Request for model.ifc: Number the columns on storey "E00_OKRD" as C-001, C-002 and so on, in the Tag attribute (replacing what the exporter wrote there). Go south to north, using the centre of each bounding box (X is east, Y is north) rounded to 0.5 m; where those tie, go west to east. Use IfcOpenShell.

First a look at what the model holds.

```python
import ifcopenshell
import ifcopenshell.util.element
import ifcopenshell.util.placement

model = ifcopenshell.open("model.ifc")
print(model.schema)
storey = next(s for s in model.by_type("IfcBuildingStorey") if s.Name == "E00_OKRD")
columns = [e for e in ifcopenshell.util.element.get_decomposition(storey) if e.is_a("IfcColumn")]
for e in sorted(columns, key=lambda e: e.id()):
    origin = ifcopenshell.util.placement.get_local_placement(e.ObjectPlacement)[:3, 3]
    print(e.id(), e.Tag, e.Name, origin.round(2) + 0.0, sep=" | ")
```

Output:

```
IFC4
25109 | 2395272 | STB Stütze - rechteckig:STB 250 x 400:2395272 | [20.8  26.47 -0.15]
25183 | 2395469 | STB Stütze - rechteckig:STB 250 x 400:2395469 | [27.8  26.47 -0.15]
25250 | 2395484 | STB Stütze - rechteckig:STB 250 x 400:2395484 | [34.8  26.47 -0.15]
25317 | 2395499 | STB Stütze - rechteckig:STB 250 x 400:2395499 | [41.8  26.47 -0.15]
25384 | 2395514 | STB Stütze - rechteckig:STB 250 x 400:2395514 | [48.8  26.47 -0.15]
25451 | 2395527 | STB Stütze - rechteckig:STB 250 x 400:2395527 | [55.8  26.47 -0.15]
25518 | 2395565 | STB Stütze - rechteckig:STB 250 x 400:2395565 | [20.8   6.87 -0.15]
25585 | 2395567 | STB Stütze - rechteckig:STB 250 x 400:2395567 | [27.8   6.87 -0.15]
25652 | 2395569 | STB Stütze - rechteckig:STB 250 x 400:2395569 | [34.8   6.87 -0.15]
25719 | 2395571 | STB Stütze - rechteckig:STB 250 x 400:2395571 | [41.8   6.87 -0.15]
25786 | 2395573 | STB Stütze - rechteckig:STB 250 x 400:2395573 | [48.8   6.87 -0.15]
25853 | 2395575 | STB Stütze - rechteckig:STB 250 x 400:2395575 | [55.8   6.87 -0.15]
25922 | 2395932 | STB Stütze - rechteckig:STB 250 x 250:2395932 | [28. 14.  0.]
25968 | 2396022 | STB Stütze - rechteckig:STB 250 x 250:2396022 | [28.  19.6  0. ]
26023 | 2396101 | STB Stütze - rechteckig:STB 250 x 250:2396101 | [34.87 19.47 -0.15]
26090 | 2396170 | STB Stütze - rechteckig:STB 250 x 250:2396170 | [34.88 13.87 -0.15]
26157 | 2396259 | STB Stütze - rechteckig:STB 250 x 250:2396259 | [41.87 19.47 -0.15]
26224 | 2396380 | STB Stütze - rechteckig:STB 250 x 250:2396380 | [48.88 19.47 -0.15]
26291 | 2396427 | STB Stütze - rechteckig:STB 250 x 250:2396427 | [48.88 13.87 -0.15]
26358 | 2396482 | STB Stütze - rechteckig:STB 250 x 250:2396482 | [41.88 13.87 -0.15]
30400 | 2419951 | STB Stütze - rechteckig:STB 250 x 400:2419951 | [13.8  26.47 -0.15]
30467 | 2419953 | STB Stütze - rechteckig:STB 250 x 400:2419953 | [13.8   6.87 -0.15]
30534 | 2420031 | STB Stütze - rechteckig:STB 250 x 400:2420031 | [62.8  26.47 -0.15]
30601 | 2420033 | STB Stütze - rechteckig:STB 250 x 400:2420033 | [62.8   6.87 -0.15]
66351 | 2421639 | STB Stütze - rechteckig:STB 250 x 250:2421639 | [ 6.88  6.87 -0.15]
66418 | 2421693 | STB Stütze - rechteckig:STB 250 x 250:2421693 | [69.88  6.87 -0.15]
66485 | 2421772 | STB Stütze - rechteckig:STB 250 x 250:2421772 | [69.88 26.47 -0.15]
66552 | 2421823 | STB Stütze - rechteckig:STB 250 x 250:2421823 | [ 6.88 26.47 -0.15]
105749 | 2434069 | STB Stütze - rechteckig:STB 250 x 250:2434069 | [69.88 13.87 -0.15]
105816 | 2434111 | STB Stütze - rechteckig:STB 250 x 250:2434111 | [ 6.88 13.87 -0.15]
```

```python
import ifcopenshell
import ifcopenshell.geom
import ifcopenshell.util.element
import ifcopenshell.util.shape

model = ifcopenshell.open("model.ifc")
settings = ifcopenshell.geom.settings()
settings.set("use-world-coords", True)


def centre(element):
    shape = ifcopenshell.geom.create_shape(settings, element)
    return ifcopenshell.util.shape.get_bbox_centroid(shape.geometry)


storey = next(s for s in model.by_type("IfcBuildingStorey") if s.Name == "E00_OKRD")
columns = [e for e in ifcopenshell.util.element.get_decomposition(storey) if e.is_a("IfcColumn")]

# Insertion points can sit at a corner or the storey origin, so sort by the geometry (in metres).
centres = {e: centre(e) for e in columns}
columns.sort(key=lambda e: (round(centres[e][1] / 0.5), centres[e][0]))

for i, e in enumerate(columns, start=1):
    number = f"C-0{i:02d}"
    e.Tag = number
    print(e.id(), number)

model.write("model_updated.ifc")
```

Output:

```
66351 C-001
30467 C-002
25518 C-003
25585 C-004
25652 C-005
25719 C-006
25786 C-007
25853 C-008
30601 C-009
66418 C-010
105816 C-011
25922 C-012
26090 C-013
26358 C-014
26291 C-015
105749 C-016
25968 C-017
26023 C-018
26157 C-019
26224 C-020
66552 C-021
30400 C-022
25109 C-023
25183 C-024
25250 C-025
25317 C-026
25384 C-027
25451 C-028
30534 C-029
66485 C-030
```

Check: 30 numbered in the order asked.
